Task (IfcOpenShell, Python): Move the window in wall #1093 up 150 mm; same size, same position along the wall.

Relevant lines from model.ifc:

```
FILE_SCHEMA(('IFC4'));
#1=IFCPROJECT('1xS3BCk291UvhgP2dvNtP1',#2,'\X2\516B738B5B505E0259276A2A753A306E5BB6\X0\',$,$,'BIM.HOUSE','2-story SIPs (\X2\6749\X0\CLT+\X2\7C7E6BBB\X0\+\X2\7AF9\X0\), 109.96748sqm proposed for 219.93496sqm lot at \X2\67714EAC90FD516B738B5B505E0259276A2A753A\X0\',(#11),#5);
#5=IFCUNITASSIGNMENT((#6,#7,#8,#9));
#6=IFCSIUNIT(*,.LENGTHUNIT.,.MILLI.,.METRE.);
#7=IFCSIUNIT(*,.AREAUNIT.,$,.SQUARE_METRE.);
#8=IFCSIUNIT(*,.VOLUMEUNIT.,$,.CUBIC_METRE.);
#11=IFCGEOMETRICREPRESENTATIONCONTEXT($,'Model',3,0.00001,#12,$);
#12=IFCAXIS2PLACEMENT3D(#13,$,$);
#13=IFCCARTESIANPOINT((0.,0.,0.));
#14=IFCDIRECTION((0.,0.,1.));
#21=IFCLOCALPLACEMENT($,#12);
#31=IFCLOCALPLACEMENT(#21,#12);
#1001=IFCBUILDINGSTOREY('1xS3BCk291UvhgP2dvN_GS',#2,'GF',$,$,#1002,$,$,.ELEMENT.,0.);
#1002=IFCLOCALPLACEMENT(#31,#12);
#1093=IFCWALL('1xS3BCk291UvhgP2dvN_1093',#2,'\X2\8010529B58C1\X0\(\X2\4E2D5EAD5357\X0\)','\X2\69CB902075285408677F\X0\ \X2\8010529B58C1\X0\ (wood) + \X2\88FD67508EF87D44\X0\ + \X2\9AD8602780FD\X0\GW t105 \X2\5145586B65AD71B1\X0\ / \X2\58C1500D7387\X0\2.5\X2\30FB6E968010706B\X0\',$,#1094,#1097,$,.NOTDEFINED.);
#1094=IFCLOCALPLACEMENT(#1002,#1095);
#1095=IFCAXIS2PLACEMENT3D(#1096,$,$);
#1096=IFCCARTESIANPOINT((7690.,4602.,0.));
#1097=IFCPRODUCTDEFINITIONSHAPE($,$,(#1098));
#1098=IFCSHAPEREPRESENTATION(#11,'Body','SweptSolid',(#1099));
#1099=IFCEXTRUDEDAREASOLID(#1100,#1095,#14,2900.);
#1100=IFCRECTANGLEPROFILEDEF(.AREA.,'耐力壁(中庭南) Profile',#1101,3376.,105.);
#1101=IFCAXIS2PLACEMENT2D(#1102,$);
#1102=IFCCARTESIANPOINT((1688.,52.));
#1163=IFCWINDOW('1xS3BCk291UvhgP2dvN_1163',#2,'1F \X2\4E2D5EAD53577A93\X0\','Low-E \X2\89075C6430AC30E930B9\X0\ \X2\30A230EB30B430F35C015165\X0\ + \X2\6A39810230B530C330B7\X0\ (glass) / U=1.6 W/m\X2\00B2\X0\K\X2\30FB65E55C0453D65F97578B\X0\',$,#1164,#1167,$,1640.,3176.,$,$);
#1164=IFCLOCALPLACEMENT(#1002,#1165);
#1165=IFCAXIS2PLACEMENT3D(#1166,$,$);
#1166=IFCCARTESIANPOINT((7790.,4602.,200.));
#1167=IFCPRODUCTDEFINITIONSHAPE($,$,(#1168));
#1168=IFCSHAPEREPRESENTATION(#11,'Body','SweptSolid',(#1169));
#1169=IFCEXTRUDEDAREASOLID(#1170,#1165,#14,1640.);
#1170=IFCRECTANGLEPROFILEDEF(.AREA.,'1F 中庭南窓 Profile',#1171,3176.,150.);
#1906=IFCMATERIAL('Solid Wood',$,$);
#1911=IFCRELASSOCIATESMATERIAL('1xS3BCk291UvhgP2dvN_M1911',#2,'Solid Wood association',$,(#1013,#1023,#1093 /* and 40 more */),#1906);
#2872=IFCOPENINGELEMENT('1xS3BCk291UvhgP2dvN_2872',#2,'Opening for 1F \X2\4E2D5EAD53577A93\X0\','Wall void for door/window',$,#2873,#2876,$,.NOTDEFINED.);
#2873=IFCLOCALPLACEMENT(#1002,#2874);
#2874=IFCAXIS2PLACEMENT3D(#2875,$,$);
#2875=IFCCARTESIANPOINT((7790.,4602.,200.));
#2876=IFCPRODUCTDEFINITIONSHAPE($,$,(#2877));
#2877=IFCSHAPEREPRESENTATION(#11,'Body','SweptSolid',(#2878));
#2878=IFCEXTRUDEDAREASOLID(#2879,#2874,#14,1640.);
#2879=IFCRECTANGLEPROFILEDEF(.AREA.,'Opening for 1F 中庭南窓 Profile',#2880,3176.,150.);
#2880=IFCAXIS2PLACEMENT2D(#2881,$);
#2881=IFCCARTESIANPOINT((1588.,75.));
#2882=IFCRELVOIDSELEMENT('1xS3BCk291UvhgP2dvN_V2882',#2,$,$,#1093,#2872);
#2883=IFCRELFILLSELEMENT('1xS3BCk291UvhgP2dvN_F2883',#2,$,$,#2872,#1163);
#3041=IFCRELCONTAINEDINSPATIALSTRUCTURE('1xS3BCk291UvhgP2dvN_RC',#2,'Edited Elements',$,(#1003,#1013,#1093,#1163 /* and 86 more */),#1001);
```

```python
import numpy as np
import ifcopenshell
import ifcopenshell.api.geometry
import ifcopenshell.util.placement
import ifcopenshell.util.unit

model = ifcopenshell.open("model.ifc")
unit_scale = ifcopenshell.util.unit.calculate_unit_scale(model)

window = model.by_guid("1xS3BCk291UvhgP2dvN_1163")
opening = window.FillsVoids[0].RelatingOpeningElement
dz = 150.0

shift = np.array([0.0, 0.0, dz])
# The window is not placed relative to its opening, so move both.
for product in (opening, window):
    matrix = ifcopenshell.util.placement.get_local_placement(product.ObjectPlacement)
    matrix[:3, 3] += shift
    ifcopenshell.api.geometry.edit_object_placement(model, product=product, matrix=matrix, is_si=False)

print(f"moved by {dz * unit_scale:+.3f} m")

model.write("model_edited.ifc")
```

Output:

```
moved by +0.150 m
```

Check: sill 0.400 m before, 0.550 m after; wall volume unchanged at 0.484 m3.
